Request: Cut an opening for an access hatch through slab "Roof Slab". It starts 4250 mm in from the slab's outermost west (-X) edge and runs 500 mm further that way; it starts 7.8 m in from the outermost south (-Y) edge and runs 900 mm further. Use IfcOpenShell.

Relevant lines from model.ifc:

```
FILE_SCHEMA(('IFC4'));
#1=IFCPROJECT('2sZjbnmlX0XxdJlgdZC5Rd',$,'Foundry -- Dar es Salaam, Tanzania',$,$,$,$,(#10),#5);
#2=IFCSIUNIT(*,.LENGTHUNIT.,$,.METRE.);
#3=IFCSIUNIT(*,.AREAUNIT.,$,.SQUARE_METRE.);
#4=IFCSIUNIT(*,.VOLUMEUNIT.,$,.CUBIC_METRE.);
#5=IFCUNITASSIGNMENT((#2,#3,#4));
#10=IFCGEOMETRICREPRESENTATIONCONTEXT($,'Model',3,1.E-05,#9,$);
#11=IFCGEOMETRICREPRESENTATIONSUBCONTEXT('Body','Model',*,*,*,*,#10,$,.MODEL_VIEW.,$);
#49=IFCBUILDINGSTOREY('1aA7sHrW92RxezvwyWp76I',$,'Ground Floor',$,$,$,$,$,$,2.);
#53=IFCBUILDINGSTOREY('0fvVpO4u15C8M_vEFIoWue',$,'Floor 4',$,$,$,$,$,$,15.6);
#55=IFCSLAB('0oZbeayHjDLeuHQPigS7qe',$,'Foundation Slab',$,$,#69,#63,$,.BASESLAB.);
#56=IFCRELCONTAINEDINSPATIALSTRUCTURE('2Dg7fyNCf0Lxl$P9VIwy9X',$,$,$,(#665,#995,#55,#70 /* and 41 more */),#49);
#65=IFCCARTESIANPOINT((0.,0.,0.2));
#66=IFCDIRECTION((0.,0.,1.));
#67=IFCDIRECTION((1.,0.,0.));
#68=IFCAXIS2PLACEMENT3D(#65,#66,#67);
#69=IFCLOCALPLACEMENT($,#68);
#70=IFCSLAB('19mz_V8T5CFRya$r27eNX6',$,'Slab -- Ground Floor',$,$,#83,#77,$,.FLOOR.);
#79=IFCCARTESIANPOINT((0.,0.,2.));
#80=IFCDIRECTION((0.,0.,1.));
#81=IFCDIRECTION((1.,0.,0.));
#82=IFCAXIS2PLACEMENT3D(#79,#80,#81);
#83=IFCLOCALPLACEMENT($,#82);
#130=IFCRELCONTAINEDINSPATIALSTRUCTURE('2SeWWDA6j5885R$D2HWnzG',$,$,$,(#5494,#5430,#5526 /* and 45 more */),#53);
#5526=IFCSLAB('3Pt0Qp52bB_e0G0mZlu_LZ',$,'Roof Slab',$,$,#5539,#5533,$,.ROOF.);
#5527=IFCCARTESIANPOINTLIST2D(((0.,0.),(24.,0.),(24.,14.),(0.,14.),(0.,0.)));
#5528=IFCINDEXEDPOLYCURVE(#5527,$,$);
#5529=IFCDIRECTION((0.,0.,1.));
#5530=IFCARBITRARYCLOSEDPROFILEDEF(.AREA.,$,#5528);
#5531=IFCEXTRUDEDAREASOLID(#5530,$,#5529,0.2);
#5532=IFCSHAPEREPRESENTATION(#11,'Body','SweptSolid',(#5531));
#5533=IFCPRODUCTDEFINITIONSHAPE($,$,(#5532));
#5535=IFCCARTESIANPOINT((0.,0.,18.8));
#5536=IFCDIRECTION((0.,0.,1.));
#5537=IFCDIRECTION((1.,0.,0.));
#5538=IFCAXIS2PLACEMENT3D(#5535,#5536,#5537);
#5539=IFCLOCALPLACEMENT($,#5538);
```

```python
import numpy as np
import ifcopenshell
import ifcopenshell.api.feature
import ifcopenshell.api.geometry
import ifcopenshell.api.root
import ifcopenshell.geom
import ifcopenshell.util.placement
import ifcopenshell.util.representation
import ifcopenshell.util.shape
import ifcopenshell.util.unit

model = ifcopenshell.open("model.ifc")
unit_scale = ifcopenshell.util.unit.calculate_unit_scale(model)
settings = ifcopenshell.geom.settings()


def volume(element):
    """Net volume in cubic metres, openings subtracted."""
    shape = ifcopenshell.geom.create_shape(settings, element)
    return ifcopenshell.util.shape.get_volume(shape.geometry)


slab = model.by_id(5526)
before = volume(slab)

# Extent in the slab's own axes, in metres. The edges named are its -X and -Y sides.
slab_shape = ifcopenshell.geom.create_shape(settings, slab)
vertices = ifcopenshell.util.shape.get_vertices(slab_shape.geometry)
x_min, y_min, bottom = vertices.min(axis=0)
top = vertices[:, 2].max()

opening = ifcopenshell.api.root.create_entity(model, ifc_class="IfcOpeningElement", name="Access hatch opening", predefined_type="OPENING")
context = ifcopenshell.util.representation.get_context(model, "Model", "Body", "MODEL_VIEW")
width, depth = 0.5, 0.9
outline = [(0.0, 0.0), (width, 0.0), (width, depth), (0.0, depth), (0.0, 0.0)]
# Overshoot both faces by 50 mm so the cut is clean.
shape = ifcopenshell.api.geometry.add_slab_representation(
    model, context=context, depth=top - bottom + 0.1, polyline=outline
)
ifcopenshell.api.geometry.assign_representation(model, product=opening, representation=shape)

matrix = ifcopenshell.util.placement.get_local_placement(slab.ObjectPlacement)
matrix[:, 3] = matrix @ np.append(np.array([x_min + 4.25, y_min + 7.8, bottom - 0.05]) / unit_scale, 1.0)
ifcopenshell.api.geometry.edit_object_placement(model, product=opening, matrix=matrix, is_si=False)
ifcopenshell.api.feature.add_feature(model, feature=opening, element=slab)

after = volume(slab)

print(f"slab volume {before:.3f} -> {after:.3f} m3")

model.write("model_edited.ifc")
```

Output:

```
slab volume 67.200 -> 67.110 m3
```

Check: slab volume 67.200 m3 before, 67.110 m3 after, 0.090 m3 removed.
